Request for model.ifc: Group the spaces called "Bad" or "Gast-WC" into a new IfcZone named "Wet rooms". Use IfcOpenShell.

First a look at what the model holds.

```python
import ifcopenshell

model = ifcopenshell.open("model.ifc")
print(model.schema)
seen = {}
for space in model.by_type("IfcSpace"):
    seen[space.LongName] = seen.get(space.LongName, 0) + 1
for name, count in sorted(seen.items(), key=str):
    print(count, "x", name)
print("zones:", [z.Name for z in model.by_type("IfcZone")][:20])
```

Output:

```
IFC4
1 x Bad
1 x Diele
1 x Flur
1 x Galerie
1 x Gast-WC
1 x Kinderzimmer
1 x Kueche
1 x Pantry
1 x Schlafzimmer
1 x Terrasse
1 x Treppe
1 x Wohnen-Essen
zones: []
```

```python
import ifcopenshell
import ifcopenshell.api.group
import ifcopenshell.api.root

model = ifcopenshell.open("model.ifc")

names = {"Bad", "Gast-WC"}
spaces = [s for s in model.by_type("IfcSpace") if s.LongName in names]

zone = ifcopenshell.api.root.create_entity(model, ifc_class="IfcZone", name="Wet rooms")
ifcopenshell.api.group.assign_group(model, products=spaces, group=zone)
print(len(spaces), "spaces in", zone.Name)

model.write("model-out.ifc")
```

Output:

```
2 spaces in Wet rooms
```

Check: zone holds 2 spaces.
